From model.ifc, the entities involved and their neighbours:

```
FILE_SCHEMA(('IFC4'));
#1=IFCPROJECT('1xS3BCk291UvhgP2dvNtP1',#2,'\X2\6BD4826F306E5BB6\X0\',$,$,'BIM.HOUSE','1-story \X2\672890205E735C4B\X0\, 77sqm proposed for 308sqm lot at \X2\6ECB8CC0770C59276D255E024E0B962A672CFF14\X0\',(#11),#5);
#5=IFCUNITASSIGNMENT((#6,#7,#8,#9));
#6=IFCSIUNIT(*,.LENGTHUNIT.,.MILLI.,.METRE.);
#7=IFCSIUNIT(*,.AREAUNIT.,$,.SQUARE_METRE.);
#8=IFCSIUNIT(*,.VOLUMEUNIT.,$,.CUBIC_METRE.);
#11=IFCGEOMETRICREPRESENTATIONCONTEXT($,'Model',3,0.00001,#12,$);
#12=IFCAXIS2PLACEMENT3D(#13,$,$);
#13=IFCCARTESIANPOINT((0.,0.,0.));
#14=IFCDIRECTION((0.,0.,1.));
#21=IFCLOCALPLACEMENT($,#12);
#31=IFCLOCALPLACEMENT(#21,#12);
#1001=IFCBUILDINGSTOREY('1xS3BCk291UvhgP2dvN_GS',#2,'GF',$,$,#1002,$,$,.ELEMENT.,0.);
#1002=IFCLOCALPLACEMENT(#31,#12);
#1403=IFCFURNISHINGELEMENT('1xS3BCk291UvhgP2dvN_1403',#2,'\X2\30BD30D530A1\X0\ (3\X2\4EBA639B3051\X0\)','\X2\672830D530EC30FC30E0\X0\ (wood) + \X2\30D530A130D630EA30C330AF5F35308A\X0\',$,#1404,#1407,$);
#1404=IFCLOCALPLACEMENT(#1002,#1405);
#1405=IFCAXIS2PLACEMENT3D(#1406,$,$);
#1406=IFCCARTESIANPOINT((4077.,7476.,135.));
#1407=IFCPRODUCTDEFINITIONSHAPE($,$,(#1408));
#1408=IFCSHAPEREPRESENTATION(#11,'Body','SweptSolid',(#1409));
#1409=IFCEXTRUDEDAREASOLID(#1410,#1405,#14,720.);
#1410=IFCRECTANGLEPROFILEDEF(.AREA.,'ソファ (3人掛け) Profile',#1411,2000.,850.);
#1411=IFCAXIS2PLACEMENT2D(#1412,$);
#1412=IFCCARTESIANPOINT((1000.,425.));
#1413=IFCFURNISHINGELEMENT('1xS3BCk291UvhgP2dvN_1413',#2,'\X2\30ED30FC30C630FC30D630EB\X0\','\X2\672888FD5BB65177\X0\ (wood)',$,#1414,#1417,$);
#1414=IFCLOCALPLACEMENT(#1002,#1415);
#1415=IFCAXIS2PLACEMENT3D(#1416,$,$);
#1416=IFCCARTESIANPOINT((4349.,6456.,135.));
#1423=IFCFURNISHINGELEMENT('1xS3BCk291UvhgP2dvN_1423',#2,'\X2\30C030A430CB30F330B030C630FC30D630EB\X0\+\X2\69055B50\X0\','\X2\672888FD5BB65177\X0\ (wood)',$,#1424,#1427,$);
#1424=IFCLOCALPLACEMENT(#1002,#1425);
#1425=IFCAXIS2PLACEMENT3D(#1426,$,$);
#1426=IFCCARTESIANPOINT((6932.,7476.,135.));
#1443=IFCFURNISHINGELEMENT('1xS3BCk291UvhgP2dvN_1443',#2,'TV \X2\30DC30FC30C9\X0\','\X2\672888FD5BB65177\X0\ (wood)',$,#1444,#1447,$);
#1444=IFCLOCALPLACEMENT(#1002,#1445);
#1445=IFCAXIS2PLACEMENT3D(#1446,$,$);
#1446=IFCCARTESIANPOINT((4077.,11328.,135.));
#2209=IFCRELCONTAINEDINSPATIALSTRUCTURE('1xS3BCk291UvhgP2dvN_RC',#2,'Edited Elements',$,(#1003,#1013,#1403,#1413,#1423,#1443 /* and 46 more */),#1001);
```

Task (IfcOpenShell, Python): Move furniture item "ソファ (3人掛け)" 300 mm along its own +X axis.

```python
import ifcopenshell
import ifcopenshell.api.geometry
import ifcopenshell.util.placement
import ifcopenshell.util.unit

model = ifcopenshell.open("model.ifc")
unit_scale = ifcopenshell.util.unit.calculate_unit_scale(model)

item = model.by_guid("1xS3BCk291UvhgP2dvN_1403")
matrix = ifcopenshell.util.placement.get_local_placement(item.ObjectPlacement)
matrix[:3, 3] += matrix[:3, 0] * 0.3 / unit_scale
ifcopenshell.api.geometry.edit_object_placement(model, product=item, matrix=matrix, is_si=False)

print(ifcopenshell.util.placement.get_local_placement(item.ObjectPlacement).round(3) + 0.0)

model.write("model_rev.ifc")
```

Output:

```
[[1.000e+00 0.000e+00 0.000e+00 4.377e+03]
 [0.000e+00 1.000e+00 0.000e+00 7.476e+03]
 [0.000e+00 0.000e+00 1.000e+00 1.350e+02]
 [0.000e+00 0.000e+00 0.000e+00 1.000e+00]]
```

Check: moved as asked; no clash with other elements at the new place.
